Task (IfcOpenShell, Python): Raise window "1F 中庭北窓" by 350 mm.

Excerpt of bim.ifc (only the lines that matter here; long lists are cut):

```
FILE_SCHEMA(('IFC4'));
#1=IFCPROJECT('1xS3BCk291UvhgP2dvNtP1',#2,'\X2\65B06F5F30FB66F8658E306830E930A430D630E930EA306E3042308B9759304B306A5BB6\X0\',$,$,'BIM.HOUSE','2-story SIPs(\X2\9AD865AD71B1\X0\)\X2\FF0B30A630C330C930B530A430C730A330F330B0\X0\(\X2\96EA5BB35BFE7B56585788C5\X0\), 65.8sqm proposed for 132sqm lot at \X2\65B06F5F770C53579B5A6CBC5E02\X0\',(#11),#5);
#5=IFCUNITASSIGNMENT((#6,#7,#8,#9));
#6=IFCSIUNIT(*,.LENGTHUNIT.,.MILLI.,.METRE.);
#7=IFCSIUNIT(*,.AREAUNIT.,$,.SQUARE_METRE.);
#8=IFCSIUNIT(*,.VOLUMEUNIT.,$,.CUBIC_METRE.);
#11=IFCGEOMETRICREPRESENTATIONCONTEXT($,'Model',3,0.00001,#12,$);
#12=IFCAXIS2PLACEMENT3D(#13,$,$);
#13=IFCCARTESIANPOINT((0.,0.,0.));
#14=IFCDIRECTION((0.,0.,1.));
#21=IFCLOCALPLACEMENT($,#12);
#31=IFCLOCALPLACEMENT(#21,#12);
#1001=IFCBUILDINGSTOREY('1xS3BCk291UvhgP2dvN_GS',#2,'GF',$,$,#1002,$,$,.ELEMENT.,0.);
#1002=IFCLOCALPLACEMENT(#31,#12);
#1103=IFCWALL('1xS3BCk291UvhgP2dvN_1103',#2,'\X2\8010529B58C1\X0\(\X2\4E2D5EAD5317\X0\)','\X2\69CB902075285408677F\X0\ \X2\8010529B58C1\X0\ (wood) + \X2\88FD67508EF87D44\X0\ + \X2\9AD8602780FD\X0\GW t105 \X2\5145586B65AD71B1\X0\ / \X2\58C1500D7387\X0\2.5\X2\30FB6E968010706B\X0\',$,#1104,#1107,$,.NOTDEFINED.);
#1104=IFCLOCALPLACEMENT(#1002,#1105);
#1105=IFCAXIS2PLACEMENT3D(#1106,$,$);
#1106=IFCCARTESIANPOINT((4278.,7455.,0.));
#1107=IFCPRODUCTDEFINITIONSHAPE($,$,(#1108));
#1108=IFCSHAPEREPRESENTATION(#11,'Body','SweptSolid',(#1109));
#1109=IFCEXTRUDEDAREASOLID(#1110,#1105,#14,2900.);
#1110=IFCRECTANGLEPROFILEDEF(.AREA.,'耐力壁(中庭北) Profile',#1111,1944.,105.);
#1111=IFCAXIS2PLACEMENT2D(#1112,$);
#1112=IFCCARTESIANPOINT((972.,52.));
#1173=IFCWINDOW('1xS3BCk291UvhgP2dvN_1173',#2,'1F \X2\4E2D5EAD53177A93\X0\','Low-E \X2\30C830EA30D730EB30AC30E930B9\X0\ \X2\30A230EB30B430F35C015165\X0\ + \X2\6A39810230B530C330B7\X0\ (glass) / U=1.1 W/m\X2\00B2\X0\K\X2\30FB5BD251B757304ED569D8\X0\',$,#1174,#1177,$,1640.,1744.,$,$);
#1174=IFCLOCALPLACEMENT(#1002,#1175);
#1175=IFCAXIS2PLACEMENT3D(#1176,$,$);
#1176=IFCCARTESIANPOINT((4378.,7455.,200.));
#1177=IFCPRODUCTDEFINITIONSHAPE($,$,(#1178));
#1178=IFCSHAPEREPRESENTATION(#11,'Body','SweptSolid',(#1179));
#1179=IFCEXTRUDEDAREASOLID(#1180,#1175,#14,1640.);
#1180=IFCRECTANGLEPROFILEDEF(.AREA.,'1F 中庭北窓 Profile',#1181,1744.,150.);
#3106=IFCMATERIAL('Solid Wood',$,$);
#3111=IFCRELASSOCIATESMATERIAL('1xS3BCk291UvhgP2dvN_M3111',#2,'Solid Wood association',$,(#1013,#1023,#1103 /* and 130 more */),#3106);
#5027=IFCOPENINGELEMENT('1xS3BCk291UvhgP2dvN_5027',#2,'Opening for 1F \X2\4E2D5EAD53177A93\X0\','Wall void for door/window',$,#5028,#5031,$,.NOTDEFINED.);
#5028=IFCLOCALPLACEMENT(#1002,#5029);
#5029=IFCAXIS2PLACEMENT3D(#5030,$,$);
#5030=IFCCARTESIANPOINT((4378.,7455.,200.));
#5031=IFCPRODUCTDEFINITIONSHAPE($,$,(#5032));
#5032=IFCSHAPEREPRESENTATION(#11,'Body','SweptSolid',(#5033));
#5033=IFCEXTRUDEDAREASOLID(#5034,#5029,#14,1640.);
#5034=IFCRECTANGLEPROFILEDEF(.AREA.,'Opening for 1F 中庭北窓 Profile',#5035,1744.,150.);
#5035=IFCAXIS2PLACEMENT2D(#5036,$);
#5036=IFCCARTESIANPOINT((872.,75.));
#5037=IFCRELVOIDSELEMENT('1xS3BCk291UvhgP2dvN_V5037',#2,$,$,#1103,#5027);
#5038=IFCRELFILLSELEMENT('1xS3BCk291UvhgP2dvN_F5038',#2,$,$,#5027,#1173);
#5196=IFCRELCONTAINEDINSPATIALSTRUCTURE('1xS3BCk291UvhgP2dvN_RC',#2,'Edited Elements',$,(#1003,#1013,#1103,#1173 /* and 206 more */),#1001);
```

```python
import numpy as np
import ifcopenshell
import ifcopenshell.api.geometry
import ifcopenshell.util.placement
import ifcopenshell.util.unit

model = ifcopenshell.open("bim.ifc")
unit_scale = ifcopenshell.util.unit.calculate_unit_scale(model)

window = model.by_guid("1xS3BCk291UvhgP2dvN_1173")
opening = window.FillsVoids[0].RelatingOpeningElement
dz = 350.0

shift = np.array([0.0, 0.0, dz])
# The window is not placed relative to its opening, so move both.
for product in (opening, window):
    matrix = ifcopenshell.util.placement.get_local_placement(product.ObjectPlacement)
    matrix[:3, 3] += shift
    ifcopenshell.api.geometry.edit_object_placement(model, product=product, matrix=matrix, is_si=False)

print(f"moved by {dz * unit_scale:+.3f} m")

model.write("bim_edited.ifc")
```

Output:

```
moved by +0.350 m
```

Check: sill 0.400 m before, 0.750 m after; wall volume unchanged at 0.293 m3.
